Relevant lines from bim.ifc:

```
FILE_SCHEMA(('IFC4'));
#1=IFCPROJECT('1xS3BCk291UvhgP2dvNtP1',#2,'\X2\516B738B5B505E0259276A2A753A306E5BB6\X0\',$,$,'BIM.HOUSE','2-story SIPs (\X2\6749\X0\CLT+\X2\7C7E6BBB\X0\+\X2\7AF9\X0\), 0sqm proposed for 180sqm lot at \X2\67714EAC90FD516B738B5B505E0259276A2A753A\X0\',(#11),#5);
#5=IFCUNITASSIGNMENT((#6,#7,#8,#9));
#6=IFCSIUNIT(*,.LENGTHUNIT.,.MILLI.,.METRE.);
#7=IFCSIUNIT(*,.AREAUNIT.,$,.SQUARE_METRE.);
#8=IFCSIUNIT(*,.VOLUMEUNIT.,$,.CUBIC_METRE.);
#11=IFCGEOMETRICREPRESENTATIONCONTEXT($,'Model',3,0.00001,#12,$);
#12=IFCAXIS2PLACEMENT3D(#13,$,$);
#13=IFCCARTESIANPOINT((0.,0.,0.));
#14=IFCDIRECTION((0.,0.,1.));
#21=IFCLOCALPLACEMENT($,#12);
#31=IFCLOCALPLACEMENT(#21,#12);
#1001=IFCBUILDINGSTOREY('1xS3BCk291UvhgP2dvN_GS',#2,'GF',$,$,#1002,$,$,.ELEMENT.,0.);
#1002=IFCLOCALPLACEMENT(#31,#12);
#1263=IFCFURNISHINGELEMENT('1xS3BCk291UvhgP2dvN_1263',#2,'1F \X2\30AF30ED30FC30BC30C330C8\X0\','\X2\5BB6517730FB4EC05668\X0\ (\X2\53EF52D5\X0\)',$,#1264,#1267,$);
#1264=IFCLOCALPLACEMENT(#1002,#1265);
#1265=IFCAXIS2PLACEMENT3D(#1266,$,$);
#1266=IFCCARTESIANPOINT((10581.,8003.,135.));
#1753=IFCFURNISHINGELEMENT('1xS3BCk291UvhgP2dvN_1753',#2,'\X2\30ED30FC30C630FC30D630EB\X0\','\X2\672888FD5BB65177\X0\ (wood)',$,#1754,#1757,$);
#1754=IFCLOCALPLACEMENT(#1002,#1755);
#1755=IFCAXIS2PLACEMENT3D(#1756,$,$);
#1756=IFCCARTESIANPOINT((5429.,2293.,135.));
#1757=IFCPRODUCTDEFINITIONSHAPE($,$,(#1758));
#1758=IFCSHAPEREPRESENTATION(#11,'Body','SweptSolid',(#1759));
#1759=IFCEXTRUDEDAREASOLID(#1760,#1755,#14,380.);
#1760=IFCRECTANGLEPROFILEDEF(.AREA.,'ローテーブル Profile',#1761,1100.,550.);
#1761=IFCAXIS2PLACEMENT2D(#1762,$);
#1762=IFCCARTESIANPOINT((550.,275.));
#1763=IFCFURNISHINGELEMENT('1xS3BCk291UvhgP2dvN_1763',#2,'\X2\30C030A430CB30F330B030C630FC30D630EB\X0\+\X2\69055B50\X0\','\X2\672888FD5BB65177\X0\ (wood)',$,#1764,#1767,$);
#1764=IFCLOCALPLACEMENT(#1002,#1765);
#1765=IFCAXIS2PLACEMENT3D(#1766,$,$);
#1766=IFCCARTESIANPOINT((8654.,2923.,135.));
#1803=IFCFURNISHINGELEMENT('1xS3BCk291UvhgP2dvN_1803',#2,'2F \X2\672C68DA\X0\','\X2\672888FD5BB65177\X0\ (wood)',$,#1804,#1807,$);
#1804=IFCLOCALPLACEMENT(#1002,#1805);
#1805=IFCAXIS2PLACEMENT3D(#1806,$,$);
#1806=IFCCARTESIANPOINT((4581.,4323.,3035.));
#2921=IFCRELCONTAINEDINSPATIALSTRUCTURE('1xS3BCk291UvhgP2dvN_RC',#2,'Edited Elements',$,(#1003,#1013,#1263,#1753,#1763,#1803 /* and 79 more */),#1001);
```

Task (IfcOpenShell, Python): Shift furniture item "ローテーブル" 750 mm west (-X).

```python
import ifcopenshell
import ifcopenshell.api.geometry
import ifcopenshell.util.placement
import ifcopenshell.util.unit

model = ifcopenshell.open("bim.ifc")
unit_scale = ifcopenshell.util.unit.calculate_unit_scale(model)

item = model.by_guid("1xS3BCk291UvhgP2dvN_1753")
matrix = ifcopenshell.util.placement.get_local_placement(item.ObjectPlacement)
matrix[0, 3] -= 0.75 / unit_scale
ifcopenshell.api.geometry.edit_object_placement(model, product=item, matrix=matrix, is_si=False)

print(ifcopenshell.util.placement.get_local_placement(item.ObjectPlacement).round(3) + 0.0)

model.write("bim_edited.ifc")
```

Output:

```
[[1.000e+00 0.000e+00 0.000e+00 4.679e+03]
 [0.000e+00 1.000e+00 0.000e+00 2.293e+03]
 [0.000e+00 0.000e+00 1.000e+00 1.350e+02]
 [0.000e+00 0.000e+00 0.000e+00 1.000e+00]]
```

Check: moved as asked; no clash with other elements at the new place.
